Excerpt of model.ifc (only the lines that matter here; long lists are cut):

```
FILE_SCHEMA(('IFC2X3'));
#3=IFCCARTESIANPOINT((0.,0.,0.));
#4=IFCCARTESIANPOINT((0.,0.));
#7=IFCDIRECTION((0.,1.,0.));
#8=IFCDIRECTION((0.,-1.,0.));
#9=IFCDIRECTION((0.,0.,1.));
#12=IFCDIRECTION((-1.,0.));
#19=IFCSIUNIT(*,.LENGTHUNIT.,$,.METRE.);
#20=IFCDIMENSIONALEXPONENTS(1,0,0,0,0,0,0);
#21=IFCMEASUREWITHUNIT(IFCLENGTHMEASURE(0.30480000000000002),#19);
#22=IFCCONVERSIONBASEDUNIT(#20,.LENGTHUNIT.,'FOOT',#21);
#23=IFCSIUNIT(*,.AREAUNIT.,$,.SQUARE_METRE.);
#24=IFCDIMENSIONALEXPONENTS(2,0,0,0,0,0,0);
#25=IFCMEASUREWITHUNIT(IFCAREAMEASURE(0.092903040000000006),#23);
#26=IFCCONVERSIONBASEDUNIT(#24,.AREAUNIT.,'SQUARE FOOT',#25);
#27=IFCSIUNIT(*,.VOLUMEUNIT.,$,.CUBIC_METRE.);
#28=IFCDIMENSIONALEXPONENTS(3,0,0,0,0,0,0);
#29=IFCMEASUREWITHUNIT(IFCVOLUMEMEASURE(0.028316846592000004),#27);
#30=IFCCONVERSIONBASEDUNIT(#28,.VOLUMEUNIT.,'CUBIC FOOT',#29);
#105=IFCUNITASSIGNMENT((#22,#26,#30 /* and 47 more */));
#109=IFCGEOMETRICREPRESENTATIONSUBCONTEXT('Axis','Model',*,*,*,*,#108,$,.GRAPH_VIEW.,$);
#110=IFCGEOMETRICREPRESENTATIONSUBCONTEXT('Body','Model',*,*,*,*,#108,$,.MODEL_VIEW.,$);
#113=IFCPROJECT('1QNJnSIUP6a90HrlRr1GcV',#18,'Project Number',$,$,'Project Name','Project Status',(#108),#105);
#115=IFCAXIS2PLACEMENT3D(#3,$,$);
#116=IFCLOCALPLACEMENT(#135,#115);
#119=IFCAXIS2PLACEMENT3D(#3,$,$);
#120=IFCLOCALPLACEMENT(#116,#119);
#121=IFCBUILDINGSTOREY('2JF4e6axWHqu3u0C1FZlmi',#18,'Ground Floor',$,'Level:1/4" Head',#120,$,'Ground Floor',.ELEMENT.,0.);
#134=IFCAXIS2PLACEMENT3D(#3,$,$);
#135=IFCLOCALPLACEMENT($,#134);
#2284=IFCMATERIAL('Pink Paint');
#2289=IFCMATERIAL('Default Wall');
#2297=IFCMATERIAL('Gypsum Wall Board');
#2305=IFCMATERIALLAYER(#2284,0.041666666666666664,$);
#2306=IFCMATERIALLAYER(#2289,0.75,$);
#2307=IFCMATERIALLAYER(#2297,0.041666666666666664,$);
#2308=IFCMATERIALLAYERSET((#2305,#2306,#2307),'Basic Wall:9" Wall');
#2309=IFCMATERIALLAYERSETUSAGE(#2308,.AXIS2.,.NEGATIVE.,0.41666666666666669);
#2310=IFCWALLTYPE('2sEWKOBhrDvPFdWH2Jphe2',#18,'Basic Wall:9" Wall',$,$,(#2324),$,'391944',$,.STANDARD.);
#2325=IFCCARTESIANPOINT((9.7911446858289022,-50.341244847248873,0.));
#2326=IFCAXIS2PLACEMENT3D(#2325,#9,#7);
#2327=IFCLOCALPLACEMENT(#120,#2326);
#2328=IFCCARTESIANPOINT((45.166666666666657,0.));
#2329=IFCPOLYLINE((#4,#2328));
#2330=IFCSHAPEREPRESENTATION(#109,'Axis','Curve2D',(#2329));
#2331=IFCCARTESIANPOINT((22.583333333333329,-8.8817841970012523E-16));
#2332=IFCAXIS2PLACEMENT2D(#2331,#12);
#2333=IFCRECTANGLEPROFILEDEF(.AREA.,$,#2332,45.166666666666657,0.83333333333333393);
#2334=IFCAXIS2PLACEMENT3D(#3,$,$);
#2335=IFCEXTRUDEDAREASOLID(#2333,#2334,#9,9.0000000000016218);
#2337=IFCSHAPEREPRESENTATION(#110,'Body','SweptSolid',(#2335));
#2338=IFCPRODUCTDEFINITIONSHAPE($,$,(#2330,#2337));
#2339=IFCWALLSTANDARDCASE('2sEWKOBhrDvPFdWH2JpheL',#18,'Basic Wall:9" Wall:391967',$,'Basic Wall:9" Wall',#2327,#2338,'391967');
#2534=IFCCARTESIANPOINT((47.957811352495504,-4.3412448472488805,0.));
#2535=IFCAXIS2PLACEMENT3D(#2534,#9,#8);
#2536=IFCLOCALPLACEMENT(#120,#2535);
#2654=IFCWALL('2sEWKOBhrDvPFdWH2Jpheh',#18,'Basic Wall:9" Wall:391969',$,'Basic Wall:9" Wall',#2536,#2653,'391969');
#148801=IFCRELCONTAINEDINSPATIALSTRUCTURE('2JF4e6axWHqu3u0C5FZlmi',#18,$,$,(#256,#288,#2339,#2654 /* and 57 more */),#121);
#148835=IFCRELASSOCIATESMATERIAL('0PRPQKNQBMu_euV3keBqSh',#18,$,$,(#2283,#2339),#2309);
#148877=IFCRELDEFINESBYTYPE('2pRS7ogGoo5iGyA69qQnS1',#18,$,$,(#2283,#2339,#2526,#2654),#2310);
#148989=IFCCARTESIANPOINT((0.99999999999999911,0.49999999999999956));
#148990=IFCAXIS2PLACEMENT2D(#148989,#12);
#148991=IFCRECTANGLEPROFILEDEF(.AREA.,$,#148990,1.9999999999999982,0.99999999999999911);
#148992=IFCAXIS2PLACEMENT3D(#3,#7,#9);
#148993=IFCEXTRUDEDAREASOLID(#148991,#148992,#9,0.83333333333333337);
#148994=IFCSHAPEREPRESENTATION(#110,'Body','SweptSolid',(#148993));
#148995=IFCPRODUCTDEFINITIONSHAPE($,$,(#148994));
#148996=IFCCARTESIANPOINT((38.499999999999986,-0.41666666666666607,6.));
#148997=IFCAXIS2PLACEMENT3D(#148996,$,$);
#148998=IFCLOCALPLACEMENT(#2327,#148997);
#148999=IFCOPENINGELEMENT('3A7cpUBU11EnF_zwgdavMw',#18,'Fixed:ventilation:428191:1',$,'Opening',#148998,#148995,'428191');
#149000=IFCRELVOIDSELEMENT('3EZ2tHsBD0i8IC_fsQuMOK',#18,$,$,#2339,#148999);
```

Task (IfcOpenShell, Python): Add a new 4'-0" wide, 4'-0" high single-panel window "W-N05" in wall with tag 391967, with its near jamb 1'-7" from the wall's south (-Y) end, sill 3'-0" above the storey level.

```python
import numpy as np
import ifcopenshell
import ifcopenshell.api.feature
import ifcopenshell.api.geometry
import ifcopenshell.api.root
import ifcopenshell.api.spatial
import ifcopenshell.api.type
import ifcopenshell.geom
import ifcopenshell.util.element
import ifcopenshell.util.placement
import ifcopenshell.util.representation
import ifcopenshell.util.shape
import ifcopenshell.util.unit

model = ifcopenshell.open("model.ifc")
unit_scale = ifcopenshell.util.unit.calculate_unit_scale(model)
settings = ifcopenshell.geom.settings()


def volume(element):
    """Net volume in cubic metres, openings subtracted."""
    shape = ifcopenshell.geom.create_shape(settings, element)
    return ifcopenshell.util.shape.get_volume(shape.geometry)


wall = model.by_guid("2sEWKOBhrDvPFdWH2JpheL")
storey = ifcopenshell.util.element.get_container(wall, ifc_class="IfcBuildingStorey")
context = ifcopenshell.util.representation.get_context(model, "Model", "Body", "MODEL_VIEW")
before = volume(wall)

width, height, from_end, sill = 1.2192, 1.2192, 0.4826, 0.9144  # metres

# The wall runs along its own X axis, and the end named is its -X end.
wall_shape = ifcopenshell.geom.create_shape(settings, wall)
x, y, z = ifcopenshell.util.shape.get_vertices(wall_shape.geometry).T
start = x.min() + from_end
face, thickness = float(y.min()), float(y.max() - y.min())
wall_matrix = ifcopenshell.util.placement.get_local_placement(wall.ObjectPlacement)
level = ifcopenshell.util.placement.get_local_placement(storey.ObjectPlacement)[2, 3]


def in_wall(x, y):
    """Placement at x, y metres in the wall's axes, at sill height."""
    matrix = wall_matrix.copy()
    matrix[:, 3] = wall_matrix @ np.array([x / unit_scale, y / unit_scale, 0.0, 1.0])
    matrix[2, 3] = level + sill / unit_scale
    return matrix


# Opening: a box that overshoots both wall faces by 50 mm.
opening = ifcopenshell.api.root.create_entity(model, ifc_class="IfcOpeningElement")
box = ifcopenshell.api.geometry.add_wall_representation(
    model, context=context, length=width, height=height, thickness=thickness + 0.1
)
ifcopenshell.api.geometry.assign_representation(model, product=opening, representation=box)
ifcopenshell.api.geometry.edit_object_placement(model, product=opening, matrix=in_wall(start, face - 0.05), is_si=False)
ifcopenshell.api.feature.add_feature(model, feature=opening, element=wall)

window = ifcopenshell.api.root.create_entity(model, ifc_class="IfcWindow", name="W-N05")
window.OverallWidth, window.OverallHeight = width / unit_scale, height / unit_scale
body = ifcopenshell.api.geometry.add_window_representation(
    model,
    context=context,
    overall_width=window.OverallWidth,
    overall_height=window.OverallHeight,
    partition_type="SINGLE_PANEL",
)
ifcopenshell.api.geometry.assign_representation(model, product=window, representation=body)
ifcopenshell.api.spatial.assign_container(model, products=[window], relating_structure=storey)
fills = ifcopenshell.api.feature.add_filling(model, opening=opening, element=window)
fills.OwnerHistory = window.OwnerHistory  # required in IFC2X3

# IFC2X3 keeps the operation on the window style.
style = ifcopenshell.api.root.create_entity(model, ifc_class="IfcWindowStyle", name="W-N05")
style.OperationType, style.ConstructionType = "SINGLE_PANEL", "NOTDEFINED"
style.ParameterTakesPrecedence = style.Sizeable = False
ifcopenshell.api.type.assign_type(model, related_objects=[window], relating_type=style)

# Centre the window in the wall's thickness.
ifcopenshell.api.geometry.edit_object_placement(model, product=window, matrix=in_wall(start, face), is_si=False)
window_shape = ifcopenshell.geom.create_shape(settings, window)
depth = ifcopenshell.util.shape.get_vertices(window_shape.geometry)[:, 1]
offset = face + thickness / 2 - (depth.min() + depth.max()) / 2
ifcopenshell.api.geometry.edit_object_placement(model, product=window, matrix=in_wall(start, offset), is_si=False)

after = volume(wall)

print(f"wall volume {before:.3f} -> {after:.3f} m3")

model.write("model_edited.ifc")
```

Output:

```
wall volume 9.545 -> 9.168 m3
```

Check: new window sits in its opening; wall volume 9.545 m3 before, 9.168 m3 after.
